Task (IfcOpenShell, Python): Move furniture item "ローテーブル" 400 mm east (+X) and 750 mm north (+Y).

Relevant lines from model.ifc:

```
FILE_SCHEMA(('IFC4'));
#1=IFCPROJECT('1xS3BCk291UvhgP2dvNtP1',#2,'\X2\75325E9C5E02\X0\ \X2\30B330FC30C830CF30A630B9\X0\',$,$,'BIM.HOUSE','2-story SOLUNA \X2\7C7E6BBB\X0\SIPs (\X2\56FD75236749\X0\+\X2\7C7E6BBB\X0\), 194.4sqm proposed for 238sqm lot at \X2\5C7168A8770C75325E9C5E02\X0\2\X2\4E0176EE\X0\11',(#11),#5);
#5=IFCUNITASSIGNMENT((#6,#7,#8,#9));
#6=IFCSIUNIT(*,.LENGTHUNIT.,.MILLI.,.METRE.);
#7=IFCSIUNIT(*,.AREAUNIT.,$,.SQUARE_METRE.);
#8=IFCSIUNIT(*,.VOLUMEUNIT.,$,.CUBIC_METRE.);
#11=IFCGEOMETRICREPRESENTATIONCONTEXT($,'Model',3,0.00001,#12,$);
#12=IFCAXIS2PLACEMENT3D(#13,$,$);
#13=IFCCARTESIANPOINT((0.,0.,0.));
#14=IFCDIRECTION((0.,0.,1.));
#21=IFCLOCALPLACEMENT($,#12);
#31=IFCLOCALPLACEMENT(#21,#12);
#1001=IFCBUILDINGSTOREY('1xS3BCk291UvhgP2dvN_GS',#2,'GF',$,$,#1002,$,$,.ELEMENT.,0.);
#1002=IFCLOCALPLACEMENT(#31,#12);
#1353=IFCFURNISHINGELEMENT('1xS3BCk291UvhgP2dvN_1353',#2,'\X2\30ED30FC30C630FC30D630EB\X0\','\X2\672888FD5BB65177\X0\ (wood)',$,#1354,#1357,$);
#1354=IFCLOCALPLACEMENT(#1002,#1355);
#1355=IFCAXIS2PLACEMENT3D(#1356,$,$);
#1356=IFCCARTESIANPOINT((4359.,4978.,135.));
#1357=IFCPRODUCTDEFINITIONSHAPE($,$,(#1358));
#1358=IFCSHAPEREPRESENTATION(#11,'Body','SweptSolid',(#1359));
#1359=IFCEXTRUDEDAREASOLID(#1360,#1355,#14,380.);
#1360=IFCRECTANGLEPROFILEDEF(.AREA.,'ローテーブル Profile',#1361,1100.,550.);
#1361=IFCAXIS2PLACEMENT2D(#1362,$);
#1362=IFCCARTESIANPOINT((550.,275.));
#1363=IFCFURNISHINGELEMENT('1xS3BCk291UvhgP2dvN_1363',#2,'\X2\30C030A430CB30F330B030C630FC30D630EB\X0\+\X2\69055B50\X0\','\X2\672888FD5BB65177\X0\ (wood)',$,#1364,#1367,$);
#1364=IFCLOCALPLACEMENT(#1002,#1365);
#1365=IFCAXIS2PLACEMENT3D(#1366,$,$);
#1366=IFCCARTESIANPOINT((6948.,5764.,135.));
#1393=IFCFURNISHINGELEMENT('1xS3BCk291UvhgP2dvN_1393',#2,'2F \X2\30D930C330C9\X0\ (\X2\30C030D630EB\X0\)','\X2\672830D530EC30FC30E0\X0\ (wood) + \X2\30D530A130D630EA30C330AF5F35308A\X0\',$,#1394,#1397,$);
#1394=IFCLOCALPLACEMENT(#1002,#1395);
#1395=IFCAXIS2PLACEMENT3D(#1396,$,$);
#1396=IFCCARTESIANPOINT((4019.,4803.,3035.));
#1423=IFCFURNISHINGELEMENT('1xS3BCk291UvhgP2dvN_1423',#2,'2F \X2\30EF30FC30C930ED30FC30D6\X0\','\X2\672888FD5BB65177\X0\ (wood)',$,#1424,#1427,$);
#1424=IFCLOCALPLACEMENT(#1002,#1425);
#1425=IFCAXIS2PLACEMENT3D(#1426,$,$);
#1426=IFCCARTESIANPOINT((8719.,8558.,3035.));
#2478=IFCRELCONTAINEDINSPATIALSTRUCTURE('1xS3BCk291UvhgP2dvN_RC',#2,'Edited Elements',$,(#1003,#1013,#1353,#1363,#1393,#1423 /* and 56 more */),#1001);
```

```python
import ifcopenshell
import ifcopenshell.api.geometry
import ifcopenshell.util.placement

model = ifcopenshell.open("model.ifc")

item = model.by_guid("1xS3BCk291UvhgP2dvN_1353")
matrix = ifcopenshell.util.placement.get_local_placement(item.ObjectPlacement)
matrix[0, 3] += 400.0
matrix[1, 3] += 750.0
ifcopenshell.api.geometry.edit_object_placement(model, product=item, matrix=matrix, is_si=False)

print(ifcopenshell.util.placement.get_local_placement(item.ObjectPlacement).round(3) + 0.0)

model.write("model_rev.ifc")
```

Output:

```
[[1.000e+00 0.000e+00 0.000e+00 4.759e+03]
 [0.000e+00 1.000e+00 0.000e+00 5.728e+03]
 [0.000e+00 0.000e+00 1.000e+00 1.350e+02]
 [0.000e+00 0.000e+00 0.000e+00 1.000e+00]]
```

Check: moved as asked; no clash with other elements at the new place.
